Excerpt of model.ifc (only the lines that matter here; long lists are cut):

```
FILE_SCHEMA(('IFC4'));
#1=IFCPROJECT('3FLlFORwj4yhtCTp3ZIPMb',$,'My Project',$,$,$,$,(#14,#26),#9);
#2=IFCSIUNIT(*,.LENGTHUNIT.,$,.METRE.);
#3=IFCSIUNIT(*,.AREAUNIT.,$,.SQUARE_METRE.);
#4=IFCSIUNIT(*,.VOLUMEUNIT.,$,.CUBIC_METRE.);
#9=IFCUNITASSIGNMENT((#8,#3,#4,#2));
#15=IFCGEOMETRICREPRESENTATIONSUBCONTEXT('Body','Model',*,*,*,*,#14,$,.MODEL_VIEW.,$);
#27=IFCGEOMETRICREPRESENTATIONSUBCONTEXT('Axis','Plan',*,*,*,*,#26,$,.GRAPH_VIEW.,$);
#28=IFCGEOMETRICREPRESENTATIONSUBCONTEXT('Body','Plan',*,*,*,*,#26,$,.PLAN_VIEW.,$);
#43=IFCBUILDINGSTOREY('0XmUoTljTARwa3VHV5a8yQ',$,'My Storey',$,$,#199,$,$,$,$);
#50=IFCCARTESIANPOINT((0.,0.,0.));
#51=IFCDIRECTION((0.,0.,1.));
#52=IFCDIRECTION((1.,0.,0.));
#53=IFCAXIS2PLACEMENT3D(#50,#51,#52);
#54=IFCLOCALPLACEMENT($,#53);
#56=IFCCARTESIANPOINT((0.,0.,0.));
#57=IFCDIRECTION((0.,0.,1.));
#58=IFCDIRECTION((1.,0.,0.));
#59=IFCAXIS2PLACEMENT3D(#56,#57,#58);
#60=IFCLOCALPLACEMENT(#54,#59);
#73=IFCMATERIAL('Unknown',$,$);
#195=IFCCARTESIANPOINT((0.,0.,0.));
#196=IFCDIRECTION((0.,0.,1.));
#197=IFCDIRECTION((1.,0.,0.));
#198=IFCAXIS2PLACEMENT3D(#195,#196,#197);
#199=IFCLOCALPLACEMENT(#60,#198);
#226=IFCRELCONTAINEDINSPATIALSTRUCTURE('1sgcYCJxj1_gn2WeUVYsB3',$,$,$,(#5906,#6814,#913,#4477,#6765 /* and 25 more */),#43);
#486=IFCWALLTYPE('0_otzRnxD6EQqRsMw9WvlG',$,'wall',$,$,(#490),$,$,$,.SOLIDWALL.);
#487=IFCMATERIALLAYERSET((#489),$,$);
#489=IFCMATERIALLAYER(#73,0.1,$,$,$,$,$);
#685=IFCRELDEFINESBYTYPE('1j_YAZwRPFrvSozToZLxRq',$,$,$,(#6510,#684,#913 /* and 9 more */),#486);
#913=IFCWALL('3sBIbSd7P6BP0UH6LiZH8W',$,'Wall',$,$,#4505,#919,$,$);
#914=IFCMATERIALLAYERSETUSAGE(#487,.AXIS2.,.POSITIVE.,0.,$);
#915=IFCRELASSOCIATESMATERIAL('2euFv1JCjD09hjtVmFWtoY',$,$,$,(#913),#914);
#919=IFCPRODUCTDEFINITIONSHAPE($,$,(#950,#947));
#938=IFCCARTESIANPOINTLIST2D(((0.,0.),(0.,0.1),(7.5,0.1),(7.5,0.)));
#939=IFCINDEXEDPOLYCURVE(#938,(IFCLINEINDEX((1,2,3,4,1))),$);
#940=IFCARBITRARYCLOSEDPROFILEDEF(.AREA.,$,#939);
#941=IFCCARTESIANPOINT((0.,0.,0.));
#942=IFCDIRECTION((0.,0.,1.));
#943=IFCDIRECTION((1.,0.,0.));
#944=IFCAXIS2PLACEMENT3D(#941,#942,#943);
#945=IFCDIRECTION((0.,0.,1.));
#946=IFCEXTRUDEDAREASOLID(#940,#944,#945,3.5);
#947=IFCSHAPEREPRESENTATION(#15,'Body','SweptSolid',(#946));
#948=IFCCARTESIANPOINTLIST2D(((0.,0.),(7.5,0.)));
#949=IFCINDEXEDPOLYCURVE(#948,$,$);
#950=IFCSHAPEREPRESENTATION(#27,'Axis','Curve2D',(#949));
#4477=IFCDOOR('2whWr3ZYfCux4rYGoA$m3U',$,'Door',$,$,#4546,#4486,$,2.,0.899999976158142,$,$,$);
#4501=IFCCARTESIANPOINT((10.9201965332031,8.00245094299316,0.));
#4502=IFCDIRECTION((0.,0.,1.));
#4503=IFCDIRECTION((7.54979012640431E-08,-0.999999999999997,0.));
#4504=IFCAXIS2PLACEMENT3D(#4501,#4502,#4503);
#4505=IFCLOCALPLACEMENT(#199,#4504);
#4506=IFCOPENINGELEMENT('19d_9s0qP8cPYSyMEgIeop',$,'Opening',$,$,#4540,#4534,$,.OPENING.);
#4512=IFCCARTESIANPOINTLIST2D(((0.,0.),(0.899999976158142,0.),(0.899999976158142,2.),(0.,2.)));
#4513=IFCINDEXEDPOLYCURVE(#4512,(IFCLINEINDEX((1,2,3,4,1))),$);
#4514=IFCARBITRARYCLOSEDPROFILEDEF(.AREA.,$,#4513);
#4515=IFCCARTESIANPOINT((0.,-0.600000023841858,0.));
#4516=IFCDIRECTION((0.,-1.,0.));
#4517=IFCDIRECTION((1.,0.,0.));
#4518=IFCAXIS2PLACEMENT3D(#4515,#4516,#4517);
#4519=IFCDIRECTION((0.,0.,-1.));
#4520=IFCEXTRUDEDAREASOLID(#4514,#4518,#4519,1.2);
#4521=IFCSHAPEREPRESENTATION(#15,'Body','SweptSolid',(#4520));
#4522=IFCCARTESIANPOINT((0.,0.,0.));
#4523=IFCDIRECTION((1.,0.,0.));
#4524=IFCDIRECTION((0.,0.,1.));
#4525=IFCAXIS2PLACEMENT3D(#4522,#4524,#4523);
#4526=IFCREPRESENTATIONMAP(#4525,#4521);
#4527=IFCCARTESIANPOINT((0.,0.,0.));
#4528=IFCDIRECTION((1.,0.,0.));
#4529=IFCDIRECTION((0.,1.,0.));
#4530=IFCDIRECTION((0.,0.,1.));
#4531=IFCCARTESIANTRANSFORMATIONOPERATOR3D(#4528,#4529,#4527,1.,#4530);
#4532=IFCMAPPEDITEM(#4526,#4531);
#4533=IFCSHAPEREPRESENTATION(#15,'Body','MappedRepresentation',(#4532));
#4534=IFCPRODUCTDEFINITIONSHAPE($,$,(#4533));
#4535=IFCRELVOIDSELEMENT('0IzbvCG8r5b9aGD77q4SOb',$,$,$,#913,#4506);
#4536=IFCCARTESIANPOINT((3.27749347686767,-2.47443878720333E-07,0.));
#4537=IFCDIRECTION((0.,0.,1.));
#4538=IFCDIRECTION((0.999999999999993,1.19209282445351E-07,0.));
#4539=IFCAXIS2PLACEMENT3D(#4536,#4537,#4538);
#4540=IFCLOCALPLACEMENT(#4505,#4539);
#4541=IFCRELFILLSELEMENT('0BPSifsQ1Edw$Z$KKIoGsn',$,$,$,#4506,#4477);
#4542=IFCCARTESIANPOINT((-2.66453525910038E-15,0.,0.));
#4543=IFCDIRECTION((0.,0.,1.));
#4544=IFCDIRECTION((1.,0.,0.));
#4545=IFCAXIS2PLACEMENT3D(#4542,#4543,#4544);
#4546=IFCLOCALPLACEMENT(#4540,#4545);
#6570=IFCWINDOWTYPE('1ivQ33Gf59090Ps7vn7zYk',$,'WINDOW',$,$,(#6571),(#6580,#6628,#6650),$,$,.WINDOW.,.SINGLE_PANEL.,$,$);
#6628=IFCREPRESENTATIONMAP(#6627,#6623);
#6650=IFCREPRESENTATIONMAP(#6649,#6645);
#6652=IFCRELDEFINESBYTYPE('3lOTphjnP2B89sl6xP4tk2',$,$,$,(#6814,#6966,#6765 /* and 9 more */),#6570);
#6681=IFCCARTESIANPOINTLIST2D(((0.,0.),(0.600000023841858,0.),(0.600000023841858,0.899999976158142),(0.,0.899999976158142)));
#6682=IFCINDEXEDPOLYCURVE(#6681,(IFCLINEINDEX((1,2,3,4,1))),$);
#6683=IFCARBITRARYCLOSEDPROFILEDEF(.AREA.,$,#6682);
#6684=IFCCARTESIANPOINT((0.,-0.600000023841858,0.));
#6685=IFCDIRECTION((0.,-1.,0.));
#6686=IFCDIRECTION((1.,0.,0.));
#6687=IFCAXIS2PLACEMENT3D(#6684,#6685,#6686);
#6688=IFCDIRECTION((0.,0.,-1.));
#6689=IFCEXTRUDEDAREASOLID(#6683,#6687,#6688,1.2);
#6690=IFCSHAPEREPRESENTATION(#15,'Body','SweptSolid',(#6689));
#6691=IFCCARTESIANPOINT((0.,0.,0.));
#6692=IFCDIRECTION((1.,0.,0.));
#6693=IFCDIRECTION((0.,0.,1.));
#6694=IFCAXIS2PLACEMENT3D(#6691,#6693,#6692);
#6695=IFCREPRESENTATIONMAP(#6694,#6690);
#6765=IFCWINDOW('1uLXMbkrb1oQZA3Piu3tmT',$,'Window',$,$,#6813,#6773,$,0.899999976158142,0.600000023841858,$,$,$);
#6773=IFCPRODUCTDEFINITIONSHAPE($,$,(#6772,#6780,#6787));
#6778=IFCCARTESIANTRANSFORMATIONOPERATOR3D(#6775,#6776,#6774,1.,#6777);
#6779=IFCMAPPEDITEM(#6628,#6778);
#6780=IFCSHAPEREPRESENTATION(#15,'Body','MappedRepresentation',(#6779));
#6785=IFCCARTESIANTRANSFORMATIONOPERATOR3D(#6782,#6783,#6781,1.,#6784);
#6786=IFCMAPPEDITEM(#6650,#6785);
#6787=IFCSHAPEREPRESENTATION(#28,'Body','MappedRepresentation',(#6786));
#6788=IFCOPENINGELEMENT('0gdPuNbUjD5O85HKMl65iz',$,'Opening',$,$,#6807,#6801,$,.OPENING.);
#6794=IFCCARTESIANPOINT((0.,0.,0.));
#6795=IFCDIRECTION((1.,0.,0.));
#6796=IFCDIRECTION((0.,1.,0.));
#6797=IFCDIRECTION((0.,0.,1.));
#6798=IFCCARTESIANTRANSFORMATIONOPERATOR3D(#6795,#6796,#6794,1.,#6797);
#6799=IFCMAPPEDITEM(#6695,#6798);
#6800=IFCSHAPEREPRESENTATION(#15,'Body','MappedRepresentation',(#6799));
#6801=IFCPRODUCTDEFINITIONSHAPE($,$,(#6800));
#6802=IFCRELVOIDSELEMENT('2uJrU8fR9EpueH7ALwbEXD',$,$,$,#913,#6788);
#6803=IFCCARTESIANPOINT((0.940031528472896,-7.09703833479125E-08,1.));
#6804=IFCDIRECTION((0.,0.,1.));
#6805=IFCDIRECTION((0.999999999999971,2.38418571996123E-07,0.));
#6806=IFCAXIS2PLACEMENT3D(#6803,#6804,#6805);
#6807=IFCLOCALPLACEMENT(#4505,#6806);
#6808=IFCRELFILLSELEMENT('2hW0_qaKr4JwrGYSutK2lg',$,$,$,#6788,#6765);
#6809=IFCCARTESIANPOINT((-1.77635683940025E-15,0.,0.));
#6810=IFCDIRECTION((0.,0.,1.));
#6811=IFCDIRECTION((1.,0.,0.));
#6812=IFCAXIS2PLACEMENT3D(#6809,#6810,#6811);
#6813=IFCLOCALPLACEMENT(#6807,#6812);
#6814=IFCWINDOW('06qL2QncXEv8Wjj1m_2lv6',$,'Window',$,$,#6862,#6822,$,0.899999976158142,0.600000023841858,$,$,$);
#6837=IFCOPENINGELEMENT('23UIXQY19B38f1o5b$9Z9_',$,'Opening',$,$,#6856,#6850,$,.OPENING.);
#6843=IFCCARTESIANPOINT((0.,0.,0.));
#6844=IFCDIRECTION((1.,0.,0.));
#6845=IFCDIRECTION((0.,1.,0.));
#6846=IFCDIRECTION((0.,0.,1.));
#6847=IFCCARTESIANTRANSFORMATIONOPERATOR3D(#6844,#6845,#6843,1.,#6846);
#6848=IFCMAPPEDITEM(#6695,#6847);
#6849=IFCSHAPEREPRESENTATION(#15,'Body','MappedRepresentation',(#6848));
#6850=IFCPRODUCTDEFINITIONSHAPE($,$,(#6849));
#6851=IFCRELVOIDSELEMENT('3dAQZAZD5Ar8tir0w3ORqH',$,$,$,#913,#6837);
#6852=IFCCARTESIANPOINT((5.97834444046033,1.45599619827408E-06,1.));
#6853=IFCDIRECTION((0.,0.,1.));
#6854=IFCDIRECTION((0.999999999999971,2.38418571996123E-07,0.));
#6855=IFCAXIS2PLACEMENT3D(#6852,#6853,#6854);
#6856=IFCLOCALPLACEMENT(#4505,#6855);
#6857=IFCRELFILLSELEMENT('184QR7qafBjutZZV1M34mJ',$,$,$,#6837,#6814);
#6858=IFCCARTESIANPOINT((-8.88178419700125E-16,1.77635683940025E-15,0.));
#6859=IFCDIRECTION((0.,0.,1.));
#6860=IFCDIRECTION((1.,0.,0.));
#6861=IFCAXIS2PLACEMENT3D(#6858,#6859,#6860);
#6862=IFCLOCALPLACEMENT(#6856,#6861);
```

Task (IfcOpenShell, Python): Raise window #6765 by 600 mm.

```python
import numpy as np
import ifcopenshell
import ifcopenshell.api.geometry
import ifcopenshell.util.placement
import ifcopenshell.util.unit

model = ifcopenshell.open("model.ifc")
unit_scale = ifcopenshell.util.unit.calculate_unit_scale(model)

window = model.by_guid("1uLXMbkrb1oQZA3Piu3tmT")
opening = window.FillsVoids[0].RelatingOpeningElement
dz = 0.6 / unit_scale

shift = np.array([0.0, 0.0, dz])
# The window is placed relative to its opening, so it follows when the opening moves.
matrix = ifcopenshell.util.placement.get_local_placement(opening.ObjectPlacement)
matrix[:3, 3] += shift
ifcopenshell.api.geometry.edit_object_placement(
    model, product=opening, matrix=matrix, is_si=False, should_transform_children=True
)

print(f"moved by {dz * unit_scale:+.3f} m")

model.write("model-out.ifc")
```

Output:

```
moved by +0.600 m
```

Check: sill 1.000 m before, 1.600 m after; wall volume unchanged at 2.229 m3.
